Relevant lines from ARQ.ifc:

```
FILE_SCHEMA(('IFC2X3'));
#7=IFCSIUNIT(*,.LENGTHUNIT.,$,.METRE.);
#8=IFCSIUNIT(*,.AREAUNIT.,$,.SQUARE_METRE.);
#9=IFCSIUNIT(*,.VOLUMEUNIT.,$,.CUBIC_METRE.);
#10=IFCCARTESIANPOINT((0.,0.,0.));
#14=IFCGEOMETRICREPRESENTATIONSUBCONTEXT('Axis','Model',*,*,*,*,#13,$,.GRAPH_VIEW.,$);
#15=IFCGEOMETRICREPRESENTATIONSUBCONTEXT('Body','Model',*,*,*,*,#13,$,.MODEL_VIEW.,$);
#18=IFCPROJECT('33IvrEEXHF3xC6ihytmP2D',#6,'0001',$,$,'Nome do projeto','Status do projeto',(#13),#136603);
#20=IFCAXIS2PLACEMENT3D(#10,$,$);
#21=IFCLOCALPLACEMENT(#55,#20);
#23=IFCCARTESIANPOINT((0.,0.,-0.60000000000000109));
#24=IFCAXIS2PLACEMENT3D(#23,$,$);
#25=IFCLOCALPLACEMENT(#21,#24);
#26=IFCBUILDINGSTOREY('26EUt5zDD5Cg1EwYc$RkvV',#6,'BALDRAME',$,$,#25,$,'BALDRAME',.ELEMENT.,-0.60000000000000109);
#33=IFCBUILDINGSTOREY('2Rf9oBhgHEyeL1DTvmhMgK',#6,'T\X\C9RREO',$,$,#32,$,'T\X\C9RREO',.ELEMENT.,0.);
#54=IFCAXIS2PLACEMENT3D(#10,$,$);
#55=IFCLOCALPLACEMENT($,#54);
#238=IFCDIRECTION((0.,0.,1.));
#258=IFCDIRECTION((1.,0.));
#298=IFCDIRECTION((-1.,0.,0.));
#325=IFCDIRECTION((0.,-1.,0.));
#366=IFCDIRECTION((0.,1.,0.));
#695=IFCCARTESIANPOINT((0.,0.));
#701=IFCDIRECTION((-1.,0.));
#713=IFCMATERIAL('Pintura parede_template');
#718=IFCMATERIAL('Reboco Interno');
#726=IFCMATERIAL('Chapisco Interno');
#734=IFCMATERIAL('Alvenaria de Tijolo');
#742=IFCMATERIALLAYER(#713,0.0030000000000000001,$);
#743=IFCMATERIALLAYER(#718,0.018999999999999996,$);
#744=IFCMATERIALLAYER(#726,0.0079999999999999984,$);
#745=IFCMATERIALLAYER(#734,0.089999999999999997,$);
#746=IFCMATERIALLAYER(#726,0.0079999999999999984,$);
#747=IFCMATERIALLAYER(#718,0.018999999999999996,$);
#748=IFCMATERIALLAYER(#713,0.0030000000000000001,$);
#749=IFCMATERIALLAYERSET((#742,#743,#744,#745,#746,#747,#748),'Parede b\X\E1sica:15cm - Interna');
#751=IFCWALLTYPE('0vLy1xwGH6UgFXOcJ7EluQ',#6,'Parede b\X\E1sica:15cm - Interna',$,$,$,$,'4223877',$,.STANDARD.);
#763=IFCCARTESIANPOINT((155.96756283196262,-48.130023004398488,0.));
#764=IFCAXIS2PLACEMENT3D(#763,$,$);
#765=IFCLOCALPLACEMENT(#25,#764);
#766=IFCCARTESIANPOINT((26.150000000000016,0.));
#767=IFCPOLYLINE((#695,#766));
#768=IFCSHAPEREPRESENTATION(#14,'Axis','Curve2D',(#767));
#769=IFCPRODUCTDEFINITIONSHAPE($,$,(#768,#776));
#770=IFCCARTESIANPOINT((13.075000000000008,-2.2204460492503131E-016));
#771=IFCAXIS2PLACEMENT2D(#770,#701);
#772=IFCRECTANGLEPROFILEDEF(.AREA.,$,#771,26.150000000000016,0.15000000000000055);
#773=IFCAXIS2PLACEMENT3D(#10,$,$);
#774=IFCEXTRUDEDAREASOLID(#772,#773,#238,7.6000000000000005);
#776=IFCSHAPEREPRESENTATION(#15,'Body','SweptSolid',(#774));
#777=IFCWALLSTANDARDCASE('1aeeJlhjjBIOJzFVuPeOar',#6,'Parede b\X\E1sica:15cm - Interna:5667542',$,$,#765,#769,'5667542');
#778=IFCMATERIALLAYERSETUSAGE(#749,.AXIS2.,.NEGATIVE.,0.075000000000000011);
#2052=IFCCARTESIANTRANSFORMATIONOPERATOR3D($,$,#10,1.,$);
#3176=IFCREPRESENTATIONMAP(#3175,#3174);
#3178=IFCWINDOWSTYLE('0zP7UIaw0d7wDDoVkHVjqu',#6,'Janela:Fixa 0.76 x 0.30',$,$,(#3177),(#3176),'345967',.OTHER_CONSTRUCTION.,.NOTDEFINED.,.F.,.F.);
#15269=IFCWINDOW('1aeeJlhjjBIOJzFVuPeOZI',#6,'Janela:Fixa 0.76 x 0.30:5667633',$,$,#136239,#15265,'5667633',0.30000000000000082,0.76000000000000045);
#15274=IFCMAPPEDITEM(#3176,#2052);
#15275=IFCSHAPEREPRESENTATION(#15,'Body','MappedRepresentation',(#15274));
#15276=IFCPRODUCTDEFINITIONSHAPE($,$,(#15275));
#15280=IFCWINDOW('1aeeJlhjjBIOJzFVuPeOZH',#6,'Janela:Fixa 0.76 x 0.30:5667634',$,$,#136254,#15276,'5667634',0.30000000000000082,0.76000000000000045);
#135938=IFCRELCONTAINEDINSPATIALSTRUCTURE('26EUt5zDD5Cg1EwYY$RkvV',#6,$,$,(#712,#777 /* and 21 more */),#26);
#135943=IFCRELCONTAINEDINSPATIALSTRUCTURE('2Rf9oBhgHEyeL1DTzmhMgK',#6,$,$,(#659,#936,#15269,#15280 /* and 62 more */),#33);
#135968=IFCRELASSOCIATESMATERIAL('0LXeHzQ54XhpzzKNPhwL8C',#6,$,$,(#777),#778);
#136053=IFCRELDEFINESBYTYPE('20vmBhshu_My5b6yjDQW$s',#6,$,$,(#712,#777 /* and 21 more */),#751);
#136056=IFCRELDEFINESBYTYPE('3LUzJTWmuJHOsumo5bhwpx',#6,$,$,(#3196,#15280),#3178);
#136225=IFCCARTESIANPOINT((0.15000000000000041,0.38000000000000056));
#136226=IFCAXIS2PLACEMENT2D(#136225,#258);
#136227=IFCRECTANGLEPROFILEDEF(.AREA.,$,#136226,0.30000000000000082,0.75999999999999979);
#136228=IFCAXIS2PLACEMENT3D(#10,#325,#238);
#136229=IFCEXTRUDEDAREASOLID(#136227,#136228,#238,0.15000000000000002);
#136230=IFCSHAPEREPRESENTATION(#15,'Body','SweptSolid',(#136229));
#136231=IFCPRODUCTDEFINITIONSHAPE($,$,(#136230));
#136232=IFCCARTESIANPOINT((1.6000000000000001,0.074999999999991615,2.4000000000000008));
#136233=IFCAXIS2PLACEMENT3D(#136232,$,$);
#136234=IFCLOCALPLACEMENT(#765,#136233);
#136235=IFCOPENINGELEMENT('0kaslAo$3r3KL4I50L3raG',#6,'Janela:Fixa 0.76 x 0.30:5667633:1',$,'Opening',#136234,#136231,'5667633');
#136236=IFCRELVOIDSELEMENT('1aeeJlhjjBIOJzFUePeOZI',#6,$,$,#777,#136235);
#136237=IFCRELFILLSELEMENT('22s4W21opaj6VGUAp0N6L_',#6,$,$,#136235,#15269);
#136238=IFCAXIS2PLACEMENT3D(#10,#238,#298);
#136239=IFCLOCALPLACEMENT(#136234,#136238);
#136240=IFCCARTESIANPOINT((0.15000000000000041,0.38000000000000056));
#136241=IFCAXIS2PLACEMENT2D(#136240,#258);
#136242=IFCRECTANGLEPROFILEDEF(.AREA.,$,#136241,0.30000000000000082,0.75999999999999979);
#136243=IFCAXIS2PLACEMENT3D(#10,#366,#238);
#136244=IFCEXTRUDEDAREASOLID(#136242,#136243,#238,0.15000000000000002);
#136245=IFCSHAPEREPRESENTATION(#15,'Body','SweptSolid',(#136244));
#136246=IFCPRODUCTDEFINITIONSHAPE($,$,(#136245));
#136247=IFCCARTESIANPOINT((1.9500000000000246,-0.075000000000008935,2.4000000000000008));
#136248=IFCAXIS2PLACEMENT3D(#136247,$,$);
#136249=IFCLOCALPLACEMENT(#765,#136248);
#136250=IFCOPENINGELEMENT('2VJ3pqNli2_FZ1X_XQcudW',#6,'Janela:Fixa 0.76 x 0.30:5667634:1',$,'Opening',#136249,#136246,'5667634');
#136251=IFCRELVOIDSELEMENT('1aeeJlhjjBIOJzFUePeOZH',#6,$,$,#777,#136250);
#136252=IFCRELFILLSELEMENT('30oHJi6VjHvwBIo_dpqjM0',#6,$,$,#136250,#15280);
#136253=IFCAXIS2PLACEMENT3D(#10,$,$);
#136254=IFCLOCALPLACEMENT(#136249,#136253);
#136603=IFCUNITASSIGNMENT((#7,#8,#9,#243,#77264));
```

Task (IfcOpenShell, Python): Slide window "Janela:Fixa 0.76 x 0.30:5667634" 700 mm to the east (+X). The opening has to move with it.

```python
import ifcopenshell
import ifcopenshell.api.geometry
import ifcopenshell.util.placement
import ifcopenshell.util.unit

model = ifcopenshell.open("ARQ.ifc")
unit_scale = ifcopenshell.util.unit.calculate_unit_scale(model)

window = model.by_guid("1aeeJlhjjBIOJzFVuPeOZH")
opening = window.FillsVoids[0].RelatingOpeningElement
wall = opening.VoidsElements[0].RelatingBuildingElement

wall_matrix = ifcopenshell.util.placement.get_local_placement(wall.ObjectPlacement)
shift = wall_matrix[:3, 0] * 0.7 / unit_scale
before = ifcopenshell.util.placement.get_local_placement(window.ObjectPlacement)[:3, 3].copy()

# The window is placed relative to its opening, so it follows when the opening moves.
matrix = ifcopenshell.util.placement.get_local_placement(opening.ObjectPlacement)
matrix[:3, 3] += shift
ifcopenshell.api.geometry.edit_object_placement(
    model, product=opening, matrix=matrix, is_si=False, should_transform_children=True
)

after = ifcopenshell.util.placement.get_local_placement(window.ObjectPlacement)[:3, 3]
print("window moved by", (after - before).round(3) + 0.0)

model.write("ARQ_v2.ifc")
```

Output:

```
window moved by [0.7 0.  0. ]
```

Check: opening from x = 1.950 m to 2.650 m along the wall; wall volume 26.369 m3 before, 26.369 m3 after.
